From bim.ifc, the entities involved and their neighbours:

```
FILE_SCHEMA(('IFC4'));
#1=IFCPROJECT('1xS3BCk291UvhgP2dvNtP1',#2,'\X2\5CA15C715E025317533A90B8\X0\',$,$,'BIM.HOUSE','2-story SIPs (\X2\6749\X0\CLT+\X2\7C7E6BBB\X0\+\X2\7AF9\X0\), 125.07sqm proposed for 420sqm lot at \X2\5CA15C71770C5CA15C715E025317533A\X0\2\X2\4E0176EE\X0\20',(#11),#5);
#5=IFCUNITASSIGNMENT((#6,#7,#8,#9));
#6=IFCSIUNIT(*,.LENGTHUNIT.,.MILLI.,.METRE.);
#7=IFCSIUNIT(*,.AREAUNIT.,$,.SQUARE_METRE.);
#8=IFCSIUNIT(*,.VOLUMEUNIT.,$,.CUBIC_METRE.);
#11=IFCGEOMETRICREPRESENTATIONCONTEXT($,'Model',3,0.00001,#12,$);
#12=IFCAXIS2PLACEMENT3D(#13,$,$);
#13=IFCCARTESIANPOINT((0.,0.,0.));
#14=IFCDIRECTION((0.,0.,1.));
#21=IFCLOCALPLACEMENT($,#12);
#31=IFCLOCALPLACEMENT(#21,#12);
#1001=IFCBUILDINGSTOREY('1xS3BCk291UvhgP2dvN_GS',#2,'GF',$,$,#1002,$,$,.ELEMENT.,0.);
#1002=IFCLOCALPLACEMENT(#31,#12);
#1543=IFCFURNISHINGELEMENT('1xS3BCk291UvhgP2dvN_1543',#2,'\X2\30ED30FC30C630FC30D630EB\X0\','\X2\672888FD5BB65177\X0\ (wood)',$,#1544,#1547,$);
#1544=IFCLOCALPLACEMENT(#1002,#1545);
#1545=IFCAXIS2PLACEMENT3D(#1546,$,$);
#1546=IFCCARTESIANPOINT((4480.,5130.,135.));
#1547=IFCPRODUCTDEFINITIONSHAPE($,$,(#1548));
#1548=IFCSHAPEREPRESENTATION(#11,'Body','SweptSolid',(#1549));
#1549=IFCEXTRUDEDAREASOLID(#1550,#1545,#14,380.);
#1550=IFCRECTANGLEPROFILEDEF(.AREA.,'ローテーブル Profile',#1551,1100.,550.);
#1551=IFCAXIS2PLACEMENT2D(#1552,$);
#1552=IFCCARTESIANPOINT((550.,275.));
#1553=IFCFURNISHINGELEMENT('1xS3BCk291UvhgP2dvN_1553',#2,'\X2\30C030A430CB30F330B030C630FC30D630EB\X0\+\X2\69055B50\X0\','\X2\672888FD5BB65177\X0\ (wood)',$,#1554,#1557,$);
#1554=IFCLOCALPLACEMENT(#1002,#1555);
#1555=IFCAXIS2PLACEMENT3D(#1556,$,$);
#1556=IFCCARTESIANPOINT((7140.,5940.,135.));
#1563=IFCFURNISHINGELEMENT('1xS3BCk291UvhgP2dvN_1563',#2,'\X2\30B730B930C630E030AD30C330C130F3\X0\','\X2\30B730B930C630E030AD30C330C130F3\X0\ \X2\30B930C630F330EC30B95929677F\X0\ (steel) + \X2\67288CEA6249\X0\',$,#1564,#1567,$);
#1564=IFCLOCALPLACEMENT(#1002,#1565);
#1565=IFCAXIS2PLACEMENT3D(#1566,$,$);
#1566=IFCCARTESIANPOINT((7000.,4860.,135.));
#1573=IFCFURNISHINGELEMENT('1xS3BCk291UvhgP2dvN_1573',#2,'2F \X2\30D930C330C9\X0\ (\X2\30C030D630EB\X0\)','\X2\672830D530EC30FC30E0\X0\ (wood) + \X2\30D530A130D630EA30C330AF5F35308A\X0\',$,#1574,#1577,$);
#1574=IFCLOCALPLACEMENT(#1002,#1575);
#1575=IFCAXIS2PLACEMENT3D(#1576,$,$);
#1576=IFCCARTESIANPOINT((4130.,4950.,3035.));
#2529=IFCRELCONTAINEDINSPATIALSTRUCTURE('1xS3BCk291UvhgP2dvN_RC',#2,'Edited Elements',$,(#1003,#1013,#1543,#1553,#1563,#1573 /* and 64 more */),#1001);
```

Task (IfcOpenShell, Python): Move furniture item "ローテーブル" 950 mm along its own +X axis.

```python
import ifcopenshell
import ifcopenshell.api.geometry
import ifcopenshell.util.placement

model = ifcopenshell.open("bim.ifc")

item = model.by_guid("1xS3BCk291UvhgP2dvN_1543")
matrix = ifcopenshell.util.placement.get_local_placement(item.ObjectPlacement)
matrix[:3, 3] += matrix[:3, 0] * 950.0
ifcopenshell.api.geometry.edit_object_placement(model, product=item, matrix=matrix, is_si=False)

print(ifcopenshell.util.placement.get_local_placement(item.ObjectPlacement).round(3) + 0.0)

model.write("bim-out.ifc")
```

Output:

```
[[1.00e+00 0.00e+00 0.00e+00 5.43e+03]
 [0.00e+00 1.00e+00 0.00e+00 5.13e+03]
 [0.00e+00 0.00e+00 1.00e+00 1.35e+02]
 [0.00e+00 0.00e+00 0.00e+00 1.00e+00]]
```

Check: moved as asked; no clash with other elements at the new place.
